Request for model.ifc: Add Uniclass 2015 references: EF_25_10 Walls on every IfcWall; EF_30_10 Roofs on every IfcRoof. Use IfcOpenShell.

First a look at what the model holds.

```python
import ifcopenshell

model = ifcopenshell.open("model.ifc")
print(model.schema)
print("classifications:", [c.Name for c in model.by_type("IfcClassification")])
for ifc_class in ("IfcDoor", "IfcRoof", "IfcStair", "IfcWall", "IfcWindow"):
    print(ifc_class, len(model.by_type(ifc_class)))
```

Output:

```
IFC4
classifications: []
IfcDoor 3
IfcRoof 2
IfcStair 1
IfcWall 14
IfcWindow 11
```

```python
import ifcopenshell
import ifcopenshell.api.classification

model = ifcopenshell.open("model.ifc")

system = ifcopenshell.api.classification.add_classification(model, classification="Uniclass 2015")

codes = {
    "IfcWall": ("EF_25_10", "Walls"),
    "IfcRoof": ("EF_30_10", "Roofs"),
}
for ifc_class, (code, name) in codes.items():
    products = model.by_type(ifc_class)
    ifcopenshell.api.classification.add_reference(
        model, products=products, classification=system, identification=code, name=name
    )
    print(code, len(products))

model.write("model_rev.ifc")
```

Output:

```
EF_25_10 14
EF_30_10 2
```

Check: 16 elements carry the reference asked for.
